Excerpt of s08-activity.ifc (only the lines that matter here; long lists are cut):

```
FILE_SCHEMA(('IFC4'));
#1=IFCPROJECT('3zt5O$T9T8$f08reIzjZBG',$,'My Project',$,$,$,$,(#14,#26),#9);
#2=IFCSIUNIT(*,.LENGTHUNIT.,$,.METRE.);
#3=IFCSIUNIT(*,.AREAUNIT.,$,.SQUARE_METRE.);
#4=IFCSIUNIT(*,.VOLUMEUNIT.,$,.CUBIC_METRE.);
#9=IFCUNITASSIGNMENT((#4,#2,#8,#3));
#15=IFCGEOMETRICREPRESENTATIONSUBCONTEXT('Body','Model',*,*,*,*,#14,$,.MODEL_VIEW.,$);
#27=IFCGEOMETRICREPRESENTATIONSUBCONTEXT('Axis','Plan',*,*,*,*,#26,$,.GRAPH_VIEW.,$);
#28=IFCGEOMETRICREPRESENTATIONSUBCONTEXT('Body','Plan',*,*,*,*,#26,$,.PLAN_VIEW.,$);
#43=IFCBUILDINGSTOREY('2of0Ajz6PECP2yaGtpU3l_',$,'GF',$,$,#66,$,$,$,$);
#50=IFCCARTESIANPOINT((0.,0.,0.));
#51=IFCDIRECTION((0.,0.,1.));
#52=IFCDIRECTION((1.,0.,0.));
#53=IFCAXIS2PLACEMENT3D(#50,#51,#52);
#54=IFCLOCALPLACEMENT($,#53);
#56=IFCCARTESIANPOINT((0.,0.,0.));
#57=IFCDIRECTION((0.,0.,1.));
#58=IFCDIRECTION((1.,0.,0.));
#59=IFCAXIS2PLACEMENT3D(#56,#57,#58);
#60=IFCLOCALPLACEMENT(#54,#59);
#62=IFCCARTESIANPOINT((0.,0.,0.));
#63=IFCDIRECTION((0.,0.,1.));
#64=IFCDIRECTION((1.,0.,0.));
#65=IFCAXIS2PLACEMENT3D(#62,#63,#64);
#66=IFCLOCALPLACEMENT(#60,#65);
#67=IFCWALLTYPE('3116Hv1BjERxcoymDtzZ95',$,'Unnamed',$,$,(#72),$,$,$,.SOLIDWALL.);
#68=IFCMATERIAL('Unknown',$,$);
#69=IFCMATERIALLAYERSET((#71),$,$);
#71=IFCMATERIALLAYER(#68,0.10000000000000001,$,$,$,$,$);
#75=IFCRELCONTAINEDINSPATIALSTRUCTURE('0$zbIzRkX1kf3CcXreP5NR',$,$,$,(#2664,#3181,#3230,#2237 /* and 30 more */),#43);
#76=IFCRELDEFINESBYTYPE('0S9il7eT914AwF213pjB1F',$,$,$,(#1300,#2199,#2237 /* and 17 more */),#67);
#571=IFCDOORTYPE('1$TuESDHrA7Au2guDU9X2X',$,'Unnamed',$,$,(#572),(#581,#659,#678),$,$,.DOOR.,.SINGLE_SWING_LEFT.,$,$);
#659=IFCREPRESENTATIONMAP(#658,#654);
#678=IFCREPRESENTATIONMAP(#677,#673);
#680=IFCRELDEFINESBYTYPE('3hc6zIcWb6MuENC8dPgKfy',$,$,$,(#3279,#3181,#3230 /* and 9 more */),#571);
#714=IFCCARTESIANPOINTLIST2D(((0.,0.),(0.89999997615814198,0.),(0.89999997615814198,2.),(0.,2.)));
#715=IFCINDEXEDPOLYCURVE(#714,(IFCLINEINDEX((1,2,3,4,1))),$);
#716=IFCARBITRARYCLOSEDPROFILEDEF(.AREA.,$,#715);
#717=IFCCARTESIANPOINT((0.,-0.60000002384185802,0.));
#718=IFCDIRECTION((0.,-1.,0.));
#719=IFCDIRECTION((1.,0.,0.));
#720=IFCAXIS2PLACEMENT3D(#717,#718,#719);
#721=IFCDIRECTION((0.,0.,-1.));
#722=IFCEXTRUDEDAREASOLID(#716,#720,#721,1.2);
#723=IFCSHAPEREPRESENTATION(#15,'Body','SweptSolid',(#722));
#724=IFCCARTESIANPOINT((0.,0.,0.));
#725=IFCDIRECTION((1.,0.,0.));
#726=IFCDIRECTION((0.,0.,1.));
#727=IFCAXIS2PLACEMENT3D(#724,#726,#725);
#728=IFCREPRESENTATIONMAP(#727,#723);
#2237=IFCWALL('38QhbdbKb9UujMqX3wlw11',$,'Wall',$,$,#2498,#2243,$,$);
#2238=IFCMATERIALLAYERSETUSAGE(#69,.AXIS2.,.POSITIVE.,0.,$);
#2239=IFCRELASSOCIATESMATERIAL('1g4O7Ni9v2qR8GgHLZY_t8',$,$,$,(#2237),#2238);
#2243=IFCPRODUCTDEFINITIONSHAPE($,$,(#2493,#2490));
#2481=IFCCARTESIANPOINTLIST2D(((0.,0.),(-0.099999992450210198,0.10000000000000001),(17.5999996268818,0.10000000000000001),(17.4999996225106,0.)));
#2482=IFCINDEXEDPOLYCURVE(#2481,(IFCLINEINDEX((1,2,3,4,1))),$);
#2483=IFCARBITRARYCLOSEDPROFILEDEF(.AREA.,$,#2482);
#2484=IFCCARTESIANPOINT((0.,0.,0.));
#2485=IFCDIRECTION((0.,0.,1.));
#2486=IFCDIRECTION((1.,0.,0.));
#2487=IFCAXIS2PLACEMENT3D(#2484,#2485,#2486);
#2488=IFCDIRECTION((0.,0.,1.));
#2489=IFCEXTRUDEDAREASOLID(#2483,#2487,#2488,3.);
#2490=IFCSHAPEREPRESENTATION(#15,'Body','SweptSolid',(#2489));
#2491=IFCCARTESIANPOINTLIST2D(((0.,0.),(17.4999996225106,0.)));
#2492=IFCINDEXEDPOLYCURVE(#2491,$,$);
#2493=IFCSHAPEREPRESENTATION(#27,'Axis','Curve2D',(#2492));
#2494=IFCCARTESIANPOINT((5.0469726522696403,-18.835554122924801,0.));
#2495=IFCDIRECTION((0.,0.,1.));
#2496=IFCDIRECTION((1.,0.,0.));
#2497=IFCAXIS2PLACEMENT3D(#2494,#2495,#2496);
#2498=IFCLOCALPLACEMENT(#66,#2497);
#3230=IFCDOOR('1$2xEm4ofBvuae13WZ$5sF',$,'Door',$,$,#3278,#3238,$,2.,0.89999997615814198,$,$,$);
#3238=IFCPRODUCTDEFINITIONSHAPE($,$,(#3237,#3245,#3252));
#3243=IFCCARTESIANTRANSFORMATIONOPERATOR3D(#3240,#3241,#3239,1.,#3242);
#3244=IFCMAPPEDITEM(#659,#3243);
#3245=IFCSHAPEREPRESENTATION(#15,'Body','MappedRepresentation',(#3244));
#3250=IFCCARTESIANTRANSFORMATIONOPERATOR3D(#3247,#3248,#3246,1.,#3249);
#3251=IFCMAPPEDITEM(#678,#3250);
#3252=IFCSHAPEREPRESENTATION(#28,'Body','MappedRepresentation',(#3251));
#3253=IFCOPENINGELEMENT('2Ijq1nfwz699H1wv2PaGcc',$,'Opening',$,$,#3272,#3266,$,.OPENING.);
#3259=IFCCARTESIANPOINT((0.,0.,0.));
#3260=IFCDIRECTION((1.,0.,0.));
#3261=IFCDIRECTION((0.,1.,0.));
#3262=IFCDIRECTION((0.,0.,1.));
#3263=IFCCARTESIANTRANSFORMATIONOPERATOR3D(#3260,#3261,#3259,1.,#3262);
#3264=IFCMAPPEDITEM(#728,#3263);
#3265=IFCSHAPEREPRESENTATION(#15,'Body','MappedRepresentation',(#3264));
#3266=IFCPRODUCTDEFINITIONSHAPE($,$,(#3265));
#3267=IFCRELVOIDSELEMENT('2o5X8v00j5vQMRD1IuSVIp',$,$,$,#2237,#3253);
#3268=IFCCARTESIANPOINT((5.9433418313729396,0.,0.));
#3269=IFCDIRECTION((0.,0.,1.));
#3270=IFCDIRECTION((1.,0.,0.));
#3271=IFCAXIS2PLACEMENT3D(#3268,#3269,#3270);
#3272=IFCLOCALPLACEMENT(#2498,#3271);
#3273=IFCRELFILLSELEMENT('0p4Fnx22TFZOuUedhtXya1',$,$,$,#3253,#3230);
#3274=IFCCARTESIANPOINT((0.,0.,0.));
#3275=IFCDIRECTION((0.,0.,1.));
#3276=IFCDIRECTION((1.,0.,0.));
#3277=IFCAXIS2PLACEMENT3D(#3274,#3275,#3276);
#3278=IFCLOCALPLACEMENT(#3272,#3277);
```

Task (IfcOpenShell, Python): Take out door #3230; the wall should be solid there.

```python
import ifcopenshell
import ifcopenshell.api.feature
import ifcopenshell.api.root
import ifcopenshell.geom
import ifcopenshell.util.shape

model = ifcopenshell.open("s08-activity.ifc")
settings = ifcopenshell.geom.settings()


def volume(element):
    """Net volume in cubic metres, openings subtracted."""
    shape = ifcopenshell.geom.create_shape(settings, element)
    return ifcopenshell.util.shape.get_volume(shape.geometry)


door = model.by_guid("1$2xEm4ofBvuae13WZ$5sF")
opening = door.FillsVoids[0].RelatingOpeningElement
wall = opening.VoidsElements[0].RelatingBuildingElement
before = volume(wall)

ifcopenshell.api.root.remove_product(model, product=door)
ifcopenshell.api.feature.remove_feature(model, feature=opening)

after = volume(wall)

print(f"wall volume {before:.3f} -> {after:.3f} m3")

model.write("s08-activity_rev.ifc")
```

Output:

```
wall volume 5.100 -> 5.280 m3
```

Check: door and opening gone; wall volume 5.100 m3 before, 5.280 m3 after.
